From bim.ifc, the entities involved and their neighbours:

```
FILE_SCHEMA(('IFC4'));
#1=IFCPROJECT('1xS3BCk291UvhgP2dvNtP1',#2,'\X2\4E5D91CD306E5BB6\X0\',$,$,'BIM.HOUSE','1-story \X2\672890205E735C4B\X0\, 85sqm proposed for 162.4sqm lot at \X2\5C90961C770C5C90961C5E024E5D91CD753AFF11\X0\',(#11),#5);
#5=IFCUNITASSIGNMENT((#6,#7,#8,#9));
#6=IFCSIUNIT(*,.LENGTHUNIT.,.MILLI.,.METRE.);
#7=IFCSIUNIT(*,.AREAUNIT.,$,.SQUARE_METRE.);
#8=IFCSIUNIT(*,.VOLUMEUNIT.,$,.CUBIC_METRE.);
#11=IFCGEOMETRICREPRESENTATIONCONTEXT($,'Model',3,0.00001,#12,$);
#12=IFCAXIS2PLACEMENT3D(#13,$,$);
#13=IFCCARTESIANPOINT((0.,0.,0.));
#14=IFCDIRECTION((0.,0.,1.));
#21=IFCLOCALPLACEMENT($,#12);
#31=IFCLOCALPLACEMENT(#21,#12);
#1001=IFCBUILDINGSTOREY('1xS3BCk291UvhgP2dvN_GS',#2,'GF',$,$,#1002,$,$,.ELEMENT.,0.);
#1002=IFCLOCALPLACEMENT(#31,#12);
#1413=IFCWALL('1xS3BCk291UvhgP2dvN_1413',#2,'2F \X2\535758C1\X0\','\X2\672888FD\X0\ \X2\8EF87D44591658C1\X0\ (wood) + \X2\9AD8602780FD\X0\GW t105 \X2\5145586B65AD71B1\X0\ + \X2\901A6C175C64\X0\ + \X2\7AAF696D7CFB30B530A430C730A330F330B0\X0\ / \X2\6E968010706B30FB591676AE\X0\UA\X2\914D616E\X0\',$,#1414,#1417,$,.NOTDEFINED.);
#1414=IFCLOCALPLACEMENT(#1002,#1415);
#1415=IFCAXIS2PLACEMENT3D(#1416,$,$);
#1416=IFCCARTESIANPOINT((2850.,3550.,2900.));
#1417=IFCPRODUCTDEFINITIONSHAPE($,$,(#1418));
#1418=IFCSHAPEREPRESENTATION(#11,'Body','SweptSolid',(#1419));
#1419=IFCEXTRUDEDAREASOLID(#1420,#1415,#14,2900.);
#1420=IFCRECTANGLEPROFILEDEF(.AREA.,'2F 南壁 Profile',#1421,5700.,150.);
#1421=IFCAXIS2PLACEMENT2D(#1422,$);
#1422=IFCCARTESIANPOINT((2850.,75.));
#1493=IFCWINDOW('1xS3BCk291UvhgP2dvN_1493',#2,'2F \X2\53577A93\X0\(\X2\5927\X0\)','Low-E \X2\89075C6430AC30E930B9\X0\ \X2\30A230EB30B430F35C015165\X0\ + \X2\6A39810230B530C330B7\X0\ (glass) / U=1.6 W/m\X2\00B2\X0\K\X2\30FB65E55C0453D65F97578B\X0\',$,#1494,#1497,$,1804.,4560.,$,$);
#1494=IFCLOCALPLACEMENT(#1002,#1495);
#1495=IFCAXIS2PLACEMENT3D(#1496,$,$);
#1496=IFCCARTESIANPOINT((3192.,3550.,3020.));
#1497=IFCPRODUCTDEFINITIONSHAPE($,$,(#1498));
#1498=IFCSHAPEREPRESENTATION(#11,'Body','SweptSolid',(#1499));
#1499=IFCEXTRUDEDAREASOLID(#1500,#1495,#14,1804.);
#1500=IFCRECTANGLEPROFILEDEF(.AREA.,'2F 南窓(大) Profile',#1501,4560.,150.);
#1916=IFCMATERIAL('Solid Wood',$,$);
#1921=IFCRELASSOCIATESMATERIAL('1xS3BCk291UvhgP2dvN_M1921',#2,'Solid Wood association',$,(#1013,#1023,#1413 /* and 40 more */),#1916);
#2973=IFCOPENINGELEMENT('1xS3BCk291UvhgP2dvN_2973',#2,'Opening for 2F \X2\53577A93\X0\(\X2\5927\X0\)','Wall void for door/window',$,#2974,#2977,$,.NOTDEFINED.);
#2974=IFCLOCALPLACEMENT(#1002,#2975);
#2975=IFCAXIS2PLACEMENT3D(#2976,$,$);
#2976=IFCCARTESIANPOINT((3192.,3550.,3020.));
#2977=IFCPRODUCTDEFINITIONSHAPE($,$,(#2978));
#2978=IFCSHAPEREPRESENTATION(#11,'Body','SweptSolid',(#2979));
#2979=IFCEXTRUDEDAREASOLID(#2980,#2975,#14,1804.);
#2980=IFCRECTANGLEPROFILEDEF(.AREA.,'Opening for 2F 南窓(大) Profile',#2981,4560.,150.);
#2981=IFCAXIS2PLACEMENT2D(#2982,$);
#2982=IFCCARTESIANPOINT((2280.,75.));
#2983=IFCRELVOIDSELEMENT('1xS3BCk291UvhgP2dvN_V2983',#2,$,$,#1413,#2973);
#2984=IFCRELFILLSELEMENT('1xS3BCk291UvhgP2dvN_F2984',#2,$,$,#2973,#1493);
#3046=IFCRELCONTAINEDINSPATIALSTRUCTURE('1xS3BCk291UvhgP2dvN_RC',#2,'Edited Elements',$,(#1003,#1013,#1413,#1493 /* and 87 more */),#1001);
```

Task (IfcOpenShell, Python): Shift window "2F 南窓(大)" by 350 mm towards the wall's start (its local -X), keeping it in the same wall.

```python
import ifcopenshell
import ifcopenshell.api.geometry
import ifcopenshell.util.placement
import ifcopenshell.util.unit

model = ifcopenshell.open("bim.ifc")
unit_scale = ifcopenshell.util.unit.calculate_unit_scale(model)

window = model.by_guid("1xS3BCk291UvhgP2dvN_1493")
opening = window.FillsVoids[0].RelatingOpeningElement
wall = opening.VoidsElements[0].RelatingBuildingElement

wall_matrix = ifcopenshell.util.placement.get_local_placement(wall.ObjectPlacement)
shift = wall_matrix[:3, 0] * -0.35 / unit_scale
before = ifcopenshell.util.placement.get_local_placement(window.ObjectPlacement)[:3, 3].copy()

# The window is not placed relative to its opening, so move both.
for product in (opening, window):
    matrix = ifcopenshell.util.placement.get_local_placement(product.ObjectPlacement)
    matrix[:3, 3] += shift
    ifcopenshell.api.geometry.edit_object_placement(model, product=product, matrix=matrix, is_si=False)

after = ifcopenshell.util.placement.get_local_placement(window.ObjectPlacement)[:3, 3]
print("window moved by", (after - before).round(3) + 0.0)

model.write("bim_updated.ifc")
```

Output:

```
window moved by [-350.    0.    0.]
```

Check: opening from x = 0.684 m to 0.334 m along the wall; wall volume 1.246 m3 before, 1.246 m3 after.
